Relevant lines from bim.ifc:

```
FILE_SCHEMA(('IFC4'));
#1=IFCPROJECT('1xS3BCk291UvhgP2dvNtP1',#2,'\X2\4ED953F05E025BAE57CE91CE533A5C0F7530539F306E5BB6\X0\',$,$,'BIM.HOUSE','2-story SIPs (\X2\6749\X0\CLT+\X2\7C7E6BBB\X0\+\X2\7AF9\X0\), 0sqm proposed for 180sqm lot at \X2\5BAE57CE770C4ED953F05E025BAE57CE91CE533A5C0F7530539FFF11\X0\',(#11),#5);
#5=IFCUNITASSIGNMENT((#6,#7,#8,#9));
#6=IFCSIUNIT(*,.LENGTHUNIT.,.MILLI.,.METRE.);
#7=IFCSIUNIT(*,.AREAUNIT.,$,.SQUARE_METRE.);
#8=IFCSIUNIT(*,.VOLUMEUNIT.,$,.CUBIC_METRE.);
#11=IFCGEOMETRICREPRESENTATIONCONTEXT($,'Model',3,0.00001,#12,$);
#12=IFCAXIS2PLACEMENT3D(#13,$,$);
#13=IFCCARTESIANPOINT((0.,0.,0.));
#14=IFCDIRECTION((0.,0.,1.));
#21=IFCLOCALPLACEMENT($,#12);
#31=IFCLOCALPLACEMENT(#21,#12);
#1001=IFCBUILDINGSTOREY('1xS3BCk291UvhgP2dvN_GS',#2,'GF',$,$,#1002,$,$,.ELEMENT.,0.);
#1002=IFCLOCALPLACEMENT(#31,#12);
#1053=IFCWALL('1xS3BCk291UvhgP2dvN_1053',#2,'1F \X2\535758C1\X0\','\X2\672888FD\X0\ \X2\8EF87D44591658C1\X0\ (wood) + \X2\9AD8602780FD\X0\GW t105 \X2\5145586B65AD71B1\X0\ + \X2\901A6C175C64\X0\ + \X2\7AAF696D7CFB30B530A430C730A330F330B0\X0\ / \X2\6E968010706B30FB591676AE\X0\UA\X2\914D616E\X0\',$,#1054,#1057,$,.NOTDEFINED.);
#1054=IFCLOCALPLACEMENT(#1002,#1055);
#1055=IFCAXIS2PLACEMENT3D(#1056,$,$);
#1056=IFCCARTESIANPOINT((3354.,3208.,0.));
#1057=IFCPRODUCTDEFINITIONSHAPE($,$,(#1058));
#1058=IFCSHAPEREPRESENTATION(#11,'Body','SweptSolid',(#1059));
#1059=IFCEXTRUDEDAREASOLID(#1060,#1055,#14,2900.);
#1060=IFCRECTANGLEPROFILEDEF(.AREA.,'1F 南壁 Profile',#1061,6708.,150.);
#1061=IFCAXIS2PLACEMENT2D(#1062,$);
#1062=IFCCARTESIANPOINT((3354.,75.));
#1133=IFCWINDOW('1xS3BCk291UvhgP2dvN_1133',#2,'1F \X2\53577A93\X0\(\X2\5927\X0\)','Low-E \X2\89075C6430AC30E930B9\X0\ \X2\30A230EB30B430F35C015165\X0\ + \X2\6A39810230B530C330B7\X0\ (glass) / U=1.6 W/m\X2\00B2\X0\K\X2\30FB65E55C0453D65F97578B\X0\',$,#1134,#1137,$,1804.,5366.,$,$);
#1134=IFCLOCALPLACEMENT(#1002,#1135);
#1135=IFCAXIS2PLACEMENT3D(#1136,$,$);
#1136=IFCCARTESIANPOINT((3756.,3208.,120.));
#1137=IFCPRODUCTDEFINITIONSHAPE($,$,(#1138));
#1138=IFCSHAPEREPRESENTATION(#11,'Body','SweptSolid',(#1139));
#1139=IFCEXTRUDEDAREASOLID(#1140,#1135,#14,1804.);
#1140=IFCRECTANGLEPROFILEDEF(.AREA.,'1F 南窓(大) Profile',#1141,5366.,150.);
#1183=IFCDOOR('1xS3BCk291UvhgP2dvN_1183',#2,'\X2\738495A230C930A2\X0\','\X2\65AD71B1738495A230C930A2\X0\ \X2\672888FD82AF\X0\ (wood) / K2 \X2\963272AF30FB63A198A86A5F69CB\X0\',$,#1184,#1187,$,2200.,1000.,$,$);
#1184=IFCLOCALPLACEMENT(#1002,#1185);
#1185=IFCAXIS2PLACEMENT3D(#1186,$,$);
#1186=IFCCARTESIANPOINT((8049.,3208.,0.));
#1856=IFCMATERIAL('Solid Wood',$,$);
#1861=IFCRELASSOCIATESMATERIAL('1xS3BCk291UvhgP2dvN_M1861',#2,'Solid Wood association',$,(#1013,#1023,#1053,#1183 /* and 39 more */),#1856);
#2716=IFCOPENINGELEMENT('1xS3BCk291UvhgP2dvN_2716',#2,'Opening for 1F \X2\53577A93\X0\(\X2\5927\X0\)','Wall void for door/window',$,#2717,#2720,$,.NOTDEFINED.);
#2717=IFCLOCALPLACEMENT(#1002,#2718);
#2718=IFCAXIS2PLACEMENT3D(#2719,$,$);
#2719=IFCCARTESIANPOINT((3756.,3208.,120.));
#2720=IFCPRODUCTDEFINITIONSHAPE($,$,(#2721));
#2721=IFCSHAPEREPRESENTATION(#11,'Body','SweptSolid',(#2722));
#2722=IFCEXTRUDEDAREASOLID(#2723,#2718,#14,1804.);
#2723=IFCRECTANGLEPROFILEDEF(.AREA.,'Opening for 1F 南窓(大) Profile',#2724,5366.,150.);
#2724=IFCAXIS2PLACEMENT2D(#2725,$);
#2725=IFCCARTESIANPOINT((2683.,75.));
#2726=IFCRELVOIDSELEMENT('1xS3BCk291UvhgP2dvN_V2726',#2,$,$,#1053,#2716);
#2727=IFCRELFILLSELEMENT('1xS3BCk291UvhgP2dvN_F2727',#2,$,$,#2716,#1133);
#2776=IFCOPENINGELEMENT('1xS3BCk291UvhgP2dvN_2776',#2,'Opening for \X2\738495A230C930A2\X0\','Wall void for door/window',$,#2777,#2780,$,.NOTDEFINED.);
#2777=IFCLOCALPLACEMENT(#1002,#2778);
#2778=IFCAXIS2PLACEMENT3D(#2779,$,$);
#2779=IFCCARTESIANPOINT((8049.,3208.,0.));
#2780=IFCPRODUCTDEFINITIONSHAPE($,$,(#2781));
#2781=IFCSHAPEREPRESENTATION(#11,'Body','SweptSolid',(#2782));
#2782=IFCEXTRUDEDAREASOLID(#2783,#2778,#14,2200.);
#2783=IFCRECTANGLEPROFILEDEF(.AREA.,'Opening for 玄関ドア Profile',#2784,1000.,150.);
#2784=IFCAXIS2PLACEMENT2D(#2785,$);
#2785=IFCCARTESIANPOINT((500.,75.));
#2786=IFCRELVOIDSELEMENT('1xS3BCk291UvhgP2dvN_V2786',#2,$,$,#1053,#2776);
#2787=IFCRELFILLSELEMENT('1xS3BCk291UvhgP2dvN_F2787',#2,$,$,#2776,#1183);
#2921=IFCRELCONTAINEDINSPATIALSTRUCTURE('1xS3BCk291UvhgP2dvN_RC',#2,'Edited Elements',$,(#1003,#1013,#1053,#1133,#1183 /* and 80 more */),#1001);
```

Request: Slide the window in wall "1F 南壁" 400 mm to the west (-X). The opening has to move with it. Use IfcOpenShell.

```python
import ifcopenshell
import ifcopenshell.api.geometry
import ifcopenshell.util.placement

model = ifcopenshell.open("bim.ifc")

window = model.by_id(1133)
opening = window.FillsVoids[0].RelatingOpeningElement
wall = opening.VoidsElements[0].RelatingBuildingElement

wall_matrix = ifcopenshell.util.placement.get_local_placement(wall.ObjectPlacement)
shift = wall_matrix[:3, 0] * -400.0
before = ifcopenshell.util.placement.get_local_placement(window.ObjectPlacement)[:3, 3].copy()

# The window is not placed relative to its opening, so move both.
for product in (opening, window):
    matrix = ifcopenshell.util.placement.get_local_placement(product.ObjectPlacement)
    matrix[:3, 3] += shift
    ifcopenshell.api.geometry.edit_object_placement(model, product=product, matrix=matrix, is_si=False)

after = ifcopenshell.util.placement.get_local_placement(window.ObjectPlacement)[:3, 3]
print("window moved by", (after - before).round(3) + 0.0)

model.write("bim-out.ifc")
```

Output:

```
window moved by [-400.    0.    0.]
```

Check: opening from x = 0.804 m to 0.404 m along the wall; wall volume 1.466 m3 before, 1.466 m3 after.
